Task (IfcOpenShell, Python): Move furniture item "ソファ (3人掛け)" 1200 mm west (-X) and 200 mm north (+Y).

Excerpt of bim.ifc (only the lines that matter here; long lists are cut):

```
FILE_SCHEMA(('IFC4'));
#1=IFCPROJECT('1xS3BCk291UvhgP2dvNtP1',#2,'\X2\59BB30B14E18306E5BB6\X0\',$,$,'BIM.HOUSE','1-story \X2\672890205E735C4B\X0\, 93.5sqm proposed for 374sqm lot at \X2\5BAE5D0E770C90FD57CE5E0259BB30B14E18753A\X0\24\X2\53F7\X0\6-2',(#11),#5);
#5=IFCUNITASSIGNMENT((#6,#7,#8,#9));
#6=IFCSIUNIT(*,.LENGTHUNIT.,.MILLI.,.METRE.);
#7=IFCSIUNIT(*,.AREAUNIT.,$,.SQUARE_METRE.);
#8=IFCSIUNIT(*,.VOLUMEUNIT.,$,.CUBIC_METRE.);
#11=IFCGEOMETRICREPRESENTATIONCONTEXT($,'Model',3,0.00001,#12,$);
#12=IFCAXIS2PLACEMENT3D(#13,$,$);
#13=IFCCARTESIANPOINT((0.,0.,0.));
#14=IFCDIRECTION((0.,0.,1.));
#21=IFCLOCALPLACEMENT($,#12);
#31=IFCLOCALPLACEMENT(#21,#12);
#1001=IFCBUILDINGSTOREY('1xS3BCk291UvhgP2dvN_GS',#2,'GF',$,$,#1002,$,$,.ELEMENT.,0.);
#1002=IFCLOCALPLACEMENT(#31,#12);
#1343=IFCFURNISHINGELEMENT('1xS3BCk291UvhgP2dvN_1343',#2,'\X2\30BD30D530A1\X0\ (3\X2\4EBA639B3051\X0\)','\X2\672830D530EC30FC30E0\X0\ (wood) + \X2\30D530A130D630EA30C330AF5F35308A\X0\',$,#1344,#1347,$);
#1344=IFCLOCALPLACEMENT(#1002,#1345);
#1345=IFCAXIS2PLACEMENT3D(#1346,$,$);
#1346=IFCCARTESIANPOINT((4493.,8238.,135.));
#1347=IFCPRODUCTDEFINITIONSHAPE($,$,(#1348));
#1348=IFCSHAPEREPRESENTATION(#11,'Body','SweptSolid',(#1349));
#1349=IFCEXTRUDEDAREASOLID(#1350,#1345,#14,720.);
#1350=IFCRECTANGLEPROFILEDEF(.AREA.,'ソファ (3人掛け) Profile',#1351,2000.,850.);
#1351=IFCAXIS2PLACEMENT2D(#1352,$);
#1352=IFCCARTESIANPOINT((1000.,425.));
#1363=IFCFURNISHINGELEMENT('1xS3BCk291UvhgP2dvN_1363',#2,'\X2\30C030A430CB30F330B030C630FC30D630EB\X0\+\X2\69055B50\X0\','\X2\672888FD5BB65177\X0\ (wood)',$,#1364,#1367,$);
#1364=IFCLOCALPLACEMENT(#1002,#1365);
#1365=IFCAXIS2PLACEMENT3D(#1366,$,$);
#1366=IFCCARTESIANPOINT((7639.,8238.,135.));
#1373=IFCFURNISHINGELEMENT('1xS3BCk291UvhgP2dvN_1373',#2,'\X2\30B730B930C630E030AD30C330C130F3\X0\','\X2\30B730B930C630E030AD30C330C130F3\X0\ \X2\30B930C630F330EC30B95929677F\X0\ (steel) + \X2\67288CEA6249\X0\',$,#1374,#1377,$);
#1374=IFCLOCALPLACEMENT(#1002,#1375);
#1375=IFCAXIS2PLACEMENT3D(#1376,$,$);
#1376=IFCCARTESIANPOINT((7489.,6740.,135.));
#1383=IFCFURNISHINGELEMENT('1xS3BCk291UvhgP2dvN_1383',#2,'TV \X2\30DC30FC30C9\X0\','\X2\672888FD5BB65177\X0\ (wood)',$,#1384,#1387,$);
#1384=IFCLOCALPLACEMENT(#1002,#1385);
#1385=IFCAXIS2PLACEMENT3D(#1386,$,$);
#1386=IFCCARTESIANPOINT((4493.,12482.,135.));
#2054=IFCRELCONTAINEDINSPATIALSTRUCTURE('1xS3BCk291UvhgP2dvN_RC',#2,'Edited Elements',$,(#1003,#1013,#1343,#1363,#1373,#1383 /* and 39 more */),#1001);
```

```python
import ifcopenshell
import ifcopenshell.api.geometry
import ifcopenshell.util.placement
import ifcopenshell.util.unit

model = ifcopenshell.open("bim.ifc")
unit_scale = ifcopenshell.util.unit.calculate_unit_scale(model)

item = model.by_guid("1xS3BCk291UvhgP2dvN_1343")
matrix = ifcopenshell.util.placement.get_local_placement(item.ObjectPlacement)
matrix[0, 3] -= 1.2 / unit_scale
matrix[1, 3] += 0.2 / unit_scale
ifcopenshell.api.geometry.edit_object_placement(model, product=item, matrix=matrix, is_si=False)

print(ifcopenshell.util.placement.get_local_placement(item.ObjectPlacement).round(3) + 0.0)

model.write("bim-out.ifc")
```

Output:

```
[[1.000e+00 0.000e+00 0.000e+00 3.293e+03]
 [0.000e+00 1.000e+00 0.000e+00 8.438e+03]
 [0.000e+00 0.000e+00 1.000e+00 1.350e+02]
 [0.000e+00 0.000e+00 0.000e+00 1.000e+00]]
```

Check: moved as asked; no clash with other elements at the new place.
